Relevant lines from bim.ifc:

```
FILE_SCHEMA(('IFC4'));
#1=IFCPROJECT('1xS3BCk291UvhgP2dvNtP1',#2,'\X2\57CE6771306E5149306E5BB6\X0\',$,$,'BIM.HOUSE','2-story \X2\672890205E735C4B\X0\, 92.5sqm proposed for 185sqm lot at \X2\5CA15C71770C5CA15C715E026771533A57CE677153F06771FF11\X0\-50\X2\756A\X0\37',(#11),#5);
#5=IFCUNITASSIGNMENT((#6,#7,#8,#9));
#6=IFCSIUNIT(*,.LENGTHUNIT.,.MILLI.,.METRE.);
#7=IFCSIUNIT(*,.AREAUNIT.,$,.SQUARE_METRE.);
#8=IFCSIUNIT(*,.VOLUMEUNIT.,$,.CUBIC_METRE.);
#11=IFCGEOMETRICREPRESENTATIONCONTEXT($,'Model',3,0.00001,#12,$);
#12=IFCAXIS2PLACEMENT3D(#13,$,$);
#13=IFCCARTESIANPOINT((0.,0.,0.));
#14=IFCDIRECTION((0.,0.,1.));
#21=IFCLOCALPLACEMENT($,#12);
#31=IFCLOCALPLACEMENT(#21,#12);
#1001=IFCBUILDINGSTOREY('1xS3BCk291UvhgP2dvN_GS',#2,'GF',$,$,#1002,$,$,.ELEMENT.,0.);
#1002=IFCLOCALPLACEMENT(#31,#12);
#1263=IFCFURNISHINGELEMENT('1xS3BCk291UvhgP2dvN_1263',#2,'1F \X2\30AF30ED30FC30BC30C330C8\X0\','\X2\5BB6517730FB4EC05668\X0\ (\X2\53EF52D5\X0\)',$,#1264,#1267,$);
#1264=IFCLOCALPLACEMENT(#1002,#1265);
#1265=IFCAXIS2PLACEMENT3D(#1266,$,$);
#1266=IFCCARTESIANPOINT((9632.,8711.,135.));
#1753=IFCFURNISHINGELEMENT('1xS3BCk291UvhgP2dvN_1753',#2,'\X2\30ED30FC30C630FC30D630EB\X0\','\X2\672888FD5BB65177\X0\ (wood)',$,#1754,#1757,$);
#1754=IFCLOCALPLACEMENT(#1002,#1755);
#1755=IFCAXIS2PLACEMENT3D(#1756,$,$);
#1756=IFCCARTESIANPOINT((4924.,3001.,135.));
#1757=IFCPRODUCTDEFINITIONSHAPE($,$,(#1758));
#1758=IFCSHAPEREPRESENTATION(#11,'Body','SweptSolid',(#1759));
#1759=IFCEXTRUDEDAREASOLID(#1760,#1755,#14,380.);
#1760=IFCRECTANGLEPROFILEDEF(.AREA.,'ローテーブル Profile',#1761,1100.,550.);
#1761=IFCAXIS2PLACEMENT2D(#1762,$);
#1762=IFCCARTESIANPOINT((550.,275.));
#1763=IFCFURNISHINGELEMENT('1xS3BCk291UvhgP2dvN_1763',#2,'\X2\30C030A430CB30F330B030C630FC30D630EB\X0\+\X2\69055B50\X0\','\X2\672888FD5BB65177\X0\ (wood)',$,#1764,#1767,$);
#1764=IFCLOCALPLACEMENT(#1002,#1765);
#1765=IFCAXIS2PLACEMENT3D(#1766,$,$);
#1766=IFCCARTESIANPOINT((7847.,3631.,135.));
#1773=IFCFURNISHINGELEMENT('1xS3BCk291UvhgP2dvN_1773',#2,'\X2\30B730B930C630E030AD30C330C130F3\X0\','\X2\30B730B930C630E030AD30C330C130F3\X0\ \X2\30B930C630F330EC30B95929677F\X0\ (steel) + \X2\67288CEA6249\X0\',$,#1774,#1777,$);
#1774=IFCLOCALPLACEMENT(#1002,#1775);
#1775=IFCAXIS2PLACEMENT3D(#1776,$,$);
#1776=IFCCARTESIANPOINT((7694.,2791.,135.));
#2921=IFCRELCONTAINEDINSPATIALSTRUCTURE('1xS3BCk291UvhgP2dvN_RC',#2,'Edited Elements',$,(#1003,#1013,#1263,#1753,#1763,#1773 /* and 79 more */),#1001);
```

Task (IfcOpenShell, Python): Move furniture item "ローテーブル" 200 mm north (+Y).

```python
import ifcopenshell
import ifcopenshell.api.geometry
import ifcopenshell.util.placement
import ifcopenshell.util.unit

model = ifcopenshell.open("bim.ifc")
unit_scale = ifcopenshell.util.unit.calculate_unit_scale(model)

item = model.by_id(1753)
matrix = ifcopenshell.util.placement.get_local_placement(item.ObjectPlacement)
matrix[1, 3] += 0.2 / unit_scale
ifcopenshell.api.geometry.edit_object_placement(model, product=item, matrix=matrix, is_si=False)

print(ifcopenshell.util.placement.get_local_placement(item.ObjectPlacement).round(3) + 0.0)

model.write("bim_updated.ifc")
```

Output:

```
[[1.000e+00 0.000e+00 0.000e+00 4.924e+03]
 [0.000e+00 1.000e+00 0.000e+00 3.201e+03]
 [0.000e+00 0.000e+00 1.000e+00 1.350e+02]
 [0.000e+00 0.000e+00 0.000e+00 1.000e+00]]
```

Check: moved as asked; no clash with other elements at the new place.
